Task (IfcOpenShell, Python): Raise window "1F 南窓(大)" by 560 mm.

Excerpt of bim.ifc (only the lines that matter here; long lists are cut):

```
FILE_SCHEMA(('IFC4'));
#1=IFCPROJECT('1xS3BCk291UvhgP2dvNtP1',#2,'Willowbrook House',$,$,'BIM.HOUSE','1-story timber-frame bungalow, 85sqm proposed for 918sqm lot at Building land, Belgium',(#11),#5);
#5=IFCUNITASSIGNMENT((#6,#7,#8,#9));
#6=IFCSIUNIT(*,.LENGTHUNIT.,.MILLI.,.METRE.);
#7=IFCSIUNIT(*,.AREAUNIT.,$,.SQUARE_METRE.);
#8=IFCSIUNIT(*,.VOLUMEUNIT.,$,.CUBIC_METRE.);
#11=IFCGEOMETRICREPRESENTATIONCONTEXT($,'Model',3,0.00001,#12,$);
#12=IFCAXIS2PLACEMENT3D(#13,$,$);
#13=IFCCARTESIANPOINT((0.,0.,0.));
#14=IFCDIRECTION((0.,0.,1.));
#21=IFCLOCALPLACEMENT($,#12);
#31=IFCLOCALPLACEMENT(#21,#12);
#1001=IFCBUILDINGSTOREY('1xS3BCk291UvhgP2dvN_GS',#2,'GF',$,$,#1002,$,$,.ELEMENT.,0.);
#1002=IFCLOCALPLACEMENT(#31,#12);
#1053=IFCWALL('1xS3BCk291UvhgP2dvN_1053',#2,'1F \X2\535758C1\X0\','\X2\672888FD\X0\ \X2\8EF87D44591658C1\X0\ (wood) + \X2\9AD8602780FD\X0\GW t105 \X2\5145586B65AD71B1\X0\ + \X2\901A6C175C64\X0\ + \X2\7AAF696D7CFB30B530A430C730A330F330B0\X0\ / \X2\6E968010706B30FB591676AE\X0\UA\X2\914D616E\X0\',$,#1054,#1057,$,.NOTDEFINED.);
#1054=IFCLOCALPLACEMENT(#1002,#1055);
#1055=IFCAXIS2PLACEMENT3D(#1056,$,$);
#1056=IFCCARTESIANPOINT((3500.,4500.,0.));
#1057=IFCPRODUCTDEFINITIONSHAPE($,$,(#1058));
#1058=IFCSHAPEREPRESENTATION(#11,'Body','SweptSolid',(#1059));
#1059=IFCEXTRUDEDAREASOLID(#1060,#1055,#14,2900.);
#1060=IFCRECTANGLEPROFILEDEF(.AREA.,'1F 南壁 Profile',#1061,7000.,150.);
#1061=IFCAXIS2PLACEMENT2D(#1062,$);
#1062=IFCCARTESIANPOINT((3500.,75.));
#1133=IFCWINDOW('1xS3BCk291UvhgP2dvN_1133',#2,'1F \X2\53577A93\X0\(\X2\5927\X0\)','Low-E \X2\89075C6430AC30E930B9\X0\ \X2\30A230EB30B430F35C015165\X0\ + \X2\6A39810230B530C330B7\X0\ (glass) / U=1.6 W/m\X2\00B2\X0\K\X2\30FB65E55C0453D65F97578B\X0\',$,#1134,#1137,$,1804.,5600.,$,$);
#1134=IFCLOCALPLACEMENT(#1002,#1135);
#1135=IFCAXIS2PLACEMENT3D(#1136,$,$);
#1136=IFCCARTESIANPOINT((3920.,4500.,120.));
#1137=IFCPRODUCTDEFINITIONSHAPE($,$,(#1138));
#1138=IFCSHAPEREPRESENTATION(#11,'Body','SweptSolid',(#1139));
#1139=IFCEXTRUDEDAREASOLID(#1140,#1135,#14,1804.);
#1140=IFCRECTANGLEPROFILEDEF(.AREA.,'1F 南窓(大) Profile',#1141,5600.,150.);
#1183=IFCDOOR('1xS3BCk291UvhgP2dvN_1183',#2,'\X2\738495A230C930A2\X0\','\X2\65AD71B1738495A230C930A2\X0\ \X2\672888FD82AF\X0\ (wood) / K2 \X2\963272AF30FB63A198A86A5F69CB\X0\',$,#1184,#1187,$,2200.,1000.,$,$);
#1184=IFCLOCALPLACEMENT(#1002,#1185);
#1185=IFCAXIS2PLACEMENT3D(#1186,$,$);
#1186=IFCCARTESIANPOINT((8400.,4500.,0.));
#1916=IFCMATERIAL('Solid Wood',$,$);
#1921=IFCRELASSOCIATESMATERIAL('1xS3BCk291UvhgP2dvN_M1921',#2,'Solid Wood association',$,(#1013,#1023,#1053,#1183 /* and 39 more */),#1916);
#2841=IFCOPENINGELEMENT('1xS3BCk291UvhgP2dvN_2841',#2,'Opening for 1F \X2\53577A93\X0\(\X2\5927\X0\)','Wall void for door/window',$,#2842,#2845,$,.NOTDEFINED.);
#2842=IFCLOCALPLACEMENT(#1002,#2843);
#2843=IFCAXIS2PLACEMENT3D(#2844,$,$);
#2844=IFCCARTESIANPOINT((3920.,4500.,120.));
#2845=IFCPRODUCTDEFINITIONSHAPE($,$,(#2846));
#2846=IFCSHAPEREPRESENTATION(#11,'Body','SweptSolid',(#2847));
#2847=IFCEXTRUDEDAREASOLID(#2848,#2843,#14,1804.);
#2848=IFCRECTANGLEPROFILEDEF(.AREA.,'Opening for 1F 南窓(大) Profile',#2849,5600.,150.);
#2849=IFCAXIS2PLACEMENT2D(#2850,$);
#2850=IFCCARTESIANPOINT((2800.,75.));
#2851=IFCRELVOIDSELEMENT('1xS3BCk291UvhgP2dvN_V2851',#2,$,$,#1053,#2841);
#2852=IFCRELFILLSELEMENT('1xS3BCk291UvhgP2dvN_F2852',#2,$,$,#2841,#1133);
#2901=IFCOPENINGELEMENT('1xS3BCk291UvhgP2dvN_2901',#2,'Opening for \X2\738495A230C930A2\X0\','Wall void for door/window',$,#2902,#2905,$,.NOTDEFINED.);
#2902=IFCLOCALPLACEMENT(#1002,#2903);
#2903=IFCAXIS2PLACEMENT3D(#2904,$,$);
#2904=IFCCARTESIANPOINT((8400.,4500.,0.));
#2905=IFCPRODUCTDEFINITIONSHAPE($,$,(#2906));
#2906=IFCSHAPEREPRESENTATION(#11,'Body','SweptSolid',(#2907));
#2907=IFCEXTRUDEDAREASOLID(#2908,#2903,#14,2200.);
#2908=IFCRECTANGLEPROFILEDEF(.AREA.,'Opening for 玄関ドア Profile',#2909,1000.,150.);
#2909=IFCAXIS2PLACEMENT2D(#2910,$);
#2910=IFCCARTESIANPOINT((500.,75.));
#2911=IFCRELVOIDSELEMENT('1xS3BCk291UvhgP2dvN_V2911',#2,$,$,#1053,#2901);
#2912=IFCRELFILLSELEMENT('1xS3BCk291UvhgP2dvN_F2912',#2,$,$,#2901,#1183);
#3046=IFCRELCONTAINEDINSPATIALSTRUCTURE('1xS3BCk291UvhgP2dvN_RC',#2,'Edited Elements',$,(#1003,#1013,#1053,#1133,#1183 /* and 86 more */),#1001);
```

```python
import numpy as np
import ifcopenshell
import ifcopenshell.api.geometry
import ifcopenshell.util.placement
import ifcopenshell.util.unit

model = ifcopenshell.open("bim.ifc")
unit_scale = ifcopenshell.util.unit.calculate_unit_scale(model)

window = model.by_guid("1xS3BCk291UvhgP2dvN_1133")
opening = window.FillsVoids[0].RelatingOpeningElement
dz = 560.0

shift = np.array([0.0, 0.0, dz])
# The window is not placed relative to its opening, so move both.
for product in (opening, window):
    matrix = ifcopenshell.util.placement.get_local_placement(product.ObjectPlacement)
    matrix[:3, 3] += shift
    ifcopenshell.api.geometry.edit_object_placement(model, product=product, matrix=matrix, is_si=False)

print(f"moved by {dz * unit_scale:+.3f} m")

model.write("bim-out.ifc")
```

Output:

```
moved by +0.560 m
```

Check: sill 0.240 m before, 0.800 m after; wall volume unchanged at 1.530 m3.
